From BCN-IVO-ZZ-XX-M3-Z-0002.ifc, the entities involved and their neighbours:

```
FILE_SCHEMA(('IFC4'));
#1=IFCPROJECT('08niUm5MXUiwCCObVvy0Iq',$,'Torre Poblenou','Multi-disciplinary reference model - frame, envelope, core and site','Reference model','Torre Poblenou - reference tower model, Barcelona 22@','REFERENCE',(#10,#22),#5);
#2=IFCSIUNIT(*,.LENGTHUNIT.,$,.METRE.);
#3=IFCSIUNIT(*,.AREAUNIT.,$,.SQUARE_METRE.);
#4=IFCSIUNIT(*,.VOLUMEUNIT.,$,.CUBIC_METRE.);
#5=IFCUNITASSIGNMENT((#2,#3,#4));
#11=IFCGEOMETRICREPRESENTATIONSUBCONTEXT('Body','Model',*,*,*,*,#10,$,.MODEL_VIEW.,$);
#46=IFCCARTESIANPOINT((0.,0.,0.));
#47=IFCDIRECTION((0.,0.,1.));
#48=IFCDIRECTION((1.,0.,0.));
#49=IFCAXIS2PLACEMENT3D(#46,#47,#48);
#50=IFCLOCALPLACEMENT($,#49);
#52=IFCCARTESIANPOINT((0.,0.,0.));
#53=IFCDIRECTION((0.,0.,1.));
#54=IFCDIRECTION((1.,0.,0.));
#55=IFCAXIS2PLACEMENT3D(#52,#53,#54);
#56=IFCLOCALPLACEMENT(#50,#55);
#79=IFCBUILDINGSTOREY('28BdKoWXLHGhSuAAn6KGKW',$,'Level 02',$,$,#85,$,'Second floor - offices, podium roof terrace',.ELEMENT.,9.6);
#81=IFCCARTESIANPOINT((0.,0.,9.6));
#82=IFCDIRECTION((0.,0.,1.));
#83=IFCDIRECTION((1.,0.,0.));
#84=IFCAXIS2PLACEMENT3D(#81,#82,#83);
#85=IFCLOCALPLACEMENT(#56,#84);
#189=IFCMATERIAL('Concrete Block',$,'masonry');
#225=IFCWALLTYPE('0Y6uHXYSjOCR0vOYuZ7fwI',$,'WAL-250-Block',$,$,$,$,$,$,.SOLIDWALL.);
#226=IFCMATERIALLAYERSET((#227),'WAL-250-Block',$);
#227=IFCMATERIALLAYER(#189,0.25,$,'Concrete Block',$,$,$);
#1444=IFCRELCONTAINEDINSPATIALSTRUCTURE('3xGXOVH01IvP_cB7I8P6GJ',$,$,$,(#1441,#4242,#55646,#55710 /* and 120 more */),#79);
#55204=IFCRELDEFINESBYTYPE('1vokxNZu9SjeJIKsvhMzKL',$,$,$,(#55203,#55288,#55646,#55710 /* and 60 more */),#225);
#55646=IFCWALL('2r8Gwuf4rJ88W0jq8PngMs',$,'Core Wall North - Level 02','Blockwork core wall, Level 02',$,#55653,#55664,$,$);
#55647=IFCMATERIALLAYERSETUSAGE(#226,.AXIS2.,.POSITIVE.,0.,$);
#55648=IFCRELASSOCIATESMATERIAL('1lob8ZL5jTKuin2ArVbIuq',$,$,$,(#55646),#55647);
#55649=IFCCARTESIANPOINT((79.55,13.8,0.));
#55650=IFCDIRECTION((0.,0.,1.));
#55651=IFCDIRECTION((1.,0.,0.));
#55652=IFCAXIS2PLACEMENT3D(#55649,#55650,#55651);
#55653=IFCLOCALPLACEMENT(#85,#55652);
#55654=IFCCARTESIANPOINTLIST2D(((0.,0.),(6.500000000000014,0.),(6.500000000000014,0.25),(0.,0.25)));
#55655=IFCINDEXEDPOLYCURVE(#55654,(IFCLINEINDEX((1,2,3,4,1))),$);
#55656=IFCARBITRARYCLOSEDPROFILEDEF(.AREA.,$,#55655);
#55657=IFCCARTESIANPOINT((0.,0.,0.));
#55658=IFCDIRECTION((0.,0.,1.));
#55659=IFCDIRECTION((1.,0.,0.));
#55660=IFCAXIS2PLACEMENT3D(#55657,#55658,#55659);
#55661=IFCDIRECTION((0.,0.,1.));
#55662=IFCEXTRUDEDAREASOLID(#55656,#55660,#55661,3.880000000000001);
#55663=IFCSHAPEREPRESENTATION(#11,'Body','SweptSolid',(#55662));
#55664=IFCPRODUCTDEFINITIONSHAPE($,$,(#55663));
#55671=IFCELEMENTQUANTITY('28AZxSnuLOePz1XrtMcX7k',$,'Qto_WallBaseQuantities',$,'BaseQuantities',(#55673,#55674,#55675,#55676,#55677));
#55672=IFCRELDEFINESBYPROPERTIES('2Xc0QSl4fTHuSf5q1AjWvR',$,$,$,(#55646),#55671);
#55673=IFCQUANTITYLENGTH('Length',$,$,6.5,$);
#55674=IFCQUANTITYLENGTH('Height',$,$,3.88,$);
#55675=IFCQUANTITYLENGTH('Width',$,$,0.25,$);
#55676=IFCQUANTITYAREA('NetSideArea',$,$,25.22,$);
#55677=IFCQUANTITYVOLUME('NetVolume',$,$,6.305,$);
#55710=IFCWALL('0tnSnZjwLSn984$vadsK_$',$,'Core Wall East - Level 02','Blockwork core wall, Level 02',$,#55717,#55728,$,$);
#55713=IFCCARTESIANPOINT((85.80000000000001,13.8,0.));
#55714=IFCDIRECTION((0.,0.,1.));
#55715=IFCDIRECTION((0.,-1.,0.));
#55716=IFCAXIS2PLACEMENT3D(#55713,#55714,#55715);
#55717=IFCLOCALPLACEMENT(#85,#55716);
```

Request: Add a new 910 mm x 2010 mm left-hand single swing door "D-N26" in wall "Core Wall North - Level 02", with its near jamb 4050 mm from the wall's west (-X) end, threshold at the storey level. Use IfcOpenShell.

```python
import numpy as np
import ifcopenshell
import ifcopenshell.api.feature
import ifcopenshell.api.geometry
import ifcopenshell.api.pset
import ifcopenshell.api.root
import ifcopenshell.api.spatial
import ifcopenshell.geom
import ifcopenshell.util.element
import ifcopenshell.util.placement
import ifcopenshell.util.representation
import ifcopenshell.util.shape
import ifcopenshell.util.unit

model = ifcopenshell.open("BCN-IVO-ZZ-XX-M3-Z-0002.ifc")
unit_scale = ifcopenshell.util.unit.calculate_unit_scale(model)
area_scale = ifcopenshell.util.unit.calculate_unit_scale(model, "AREAUNIT")
volume_scale = ifcopenshell.util.unit.calculate_unit_scale(model, "VOLUMEUNIT")
settings = ifcopenshell.geom.settings()


def volume(element):
    """Net volume in cubic metres, openings subtracted."""
    shape = ifcopenshell.geom.create_shape(settings, element)
    return ifcopenshell.util.shape.get_volume(shape.geometry)


wall = model.by_id(55646)
storey = ifcopenshell.util.element.get_container(wall, ifc_class="IfcBuildingStorey")
context = ifcopenshell.util.representation.get_context(model, "Model", "Body", "MODEL_VIEW")
before = volume(wall)

width, height, from_end, sill = 0.91, 2.01, 4.05, 0.0  # metres

# The wall runs along its own X axis, and the end named is its -X end.
wall_shape = ifcopenshell.geom.create_shape(settings, wall)
x, y, z = ifcopenshell.util.shape.get_vertices(wall_shape.geometry).T
start = x.min() + from_end
face, thickness = float(y.min()), float(y.max() - y.min())
wall_matrix = ifcopenshell.util.placement.get_local_placement(wall.ObjectPlacement)
level = ifcopenshell.util.placement.get_local_placement(storey.ObjectPlacement)[2, 3]


def in_wall(x, y):
    """Placement at x, y metres in the wall's axes, at sill height."""
    matrix = wall_matrix.copy()
    matrix[:, 3] = wall_matrix @ np.array([x / unit_scale, y / unit_scale, 0.0, 1.0])
    matrix[2, 3] = level + sill / unit_scale
    return matrix


# Opening: a box that overshoots both wall faces by 50 mm.
opening = ifcopenshell.api.root.create_entity(model, ifc_class="IfcOpeningElement", predefined_type="OPENING")
box = ifcopenshell.api.geometry.add_wall_representation(
    model, context=context, length=width, height=height, thickness=thickness + 0.1
)
ifcopenshell.api.geometry.assign_representation(model, product=opening, representation=box)
ifcopenshell.api.geometry.edit_object_placement(model, product=opening, matrix=in_wall(start, face - 0.05), is_si=False)
ifcopenshell.api.feature.add_feature(model, feature=opening, element=wall)

door = ifcopenshell.api.root.create_entity(model, ifc_class="IfcDoor", name="D-N26", predefined_type="DOOR")
door.OverallWidth, door.OverallHeight = width / unit_scale, height / unit_scale
door.OperationType = "SINGLE_SWING_LEFT"
body = ifcopenshell.api.geometry.add_door_representation(
    model,
    context=context,
    overall_width=door.OverallWidth,
    overall_height=door.OverallHeight,
    operation_type="SINGLE_SWING_LEFT",
    lining_properties={"LiningDepth": thickness / unit_scale, "ThresholdDepth": thickness / unit_scale},
)
ifcopenshell.api.geometry.assign_representation(model, product=door, representation=body)
ifcopenshell.api.spatial.assign_container(model, products=[door], relating_structure=storey)
ifcopenshell.api.feature.add_filling(model, opening=opening, element=door)

# The lining spans the wall, so the door starts at the wall face.
ifcopenshell.api.geometry.edit_object_placement(model, product=door, matrix=in_wall(start, face), is_si=False)

after = volume(wall)

# Update the wall's stored quantities.
qto = model.by_id(ifcopenshell.util.element.get_pset(wall, "Qto_WallBaseQuantities", should_inherit=False)["id"])
ifcopenshell.api.pset.edit_qto(model, qto=qto, properties={
    "NetSideArea": after / thickness / area_scale,
    "NetVolume": after / volume_scale,
})

print(f"wall volume {before:.3f} -> {after:.3f} m3")

model.write("BCN-IVO-ZZ-XX-M3-Z-0002_v2.ifc")
```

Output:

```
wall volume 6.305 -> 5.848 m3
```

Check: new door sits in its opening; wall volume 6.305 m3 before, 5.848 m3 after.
